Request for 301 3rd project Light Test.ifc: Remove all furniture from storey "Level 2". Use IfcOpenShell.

First a look at what the model holds.

```python
import ifcopenshell
import ifcopenshell.util.element

model = ifcopenshell.open("301 3rd project Light Test.ifc")
print(model.schema)
storey = next(s for s in model.by_type("IfcBuildingStorey") if s.Name == "Level 2")
furniture = [e for e in ifcopenshell.util.element.get_decomposition(storey) if e.is_a("IfcFurnishingElement")]
seen = {}
for e in furniture:
    element_type = ifcopenshell.util.element.get_type(e)
    name = element_type.Name if element_type not in (None, e) else None
    seen[name] = seen.get(name, 0) + 1
for name, count in sorted(seen.items(), key=str):
    print(count, "x", name)
```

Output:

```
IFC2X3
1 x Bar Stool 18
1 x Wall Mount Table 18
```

```python
import ifcopenshell
import ifcopenshell.api.root
import ifcopenshell.util.element

model = ifcopenshell.open("301 3rd project Light Test.ifc")

storey = next(s for s in model.by_type("IfcBuildingStorey") if s.Name == "Level 2")
furniture = [e for e in ifcopenshell.util.element.get_decomposition(storey) if e.is_a("IfcFurnishingElement")]

for e in furniture:
    ifcopenshell.api.root.remove_product(model, product=e)
print(len(furniture), "removed")

model.write("301 3rd project Light Test_updated.ifc")
```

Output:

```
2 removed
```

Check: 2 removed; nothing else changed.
